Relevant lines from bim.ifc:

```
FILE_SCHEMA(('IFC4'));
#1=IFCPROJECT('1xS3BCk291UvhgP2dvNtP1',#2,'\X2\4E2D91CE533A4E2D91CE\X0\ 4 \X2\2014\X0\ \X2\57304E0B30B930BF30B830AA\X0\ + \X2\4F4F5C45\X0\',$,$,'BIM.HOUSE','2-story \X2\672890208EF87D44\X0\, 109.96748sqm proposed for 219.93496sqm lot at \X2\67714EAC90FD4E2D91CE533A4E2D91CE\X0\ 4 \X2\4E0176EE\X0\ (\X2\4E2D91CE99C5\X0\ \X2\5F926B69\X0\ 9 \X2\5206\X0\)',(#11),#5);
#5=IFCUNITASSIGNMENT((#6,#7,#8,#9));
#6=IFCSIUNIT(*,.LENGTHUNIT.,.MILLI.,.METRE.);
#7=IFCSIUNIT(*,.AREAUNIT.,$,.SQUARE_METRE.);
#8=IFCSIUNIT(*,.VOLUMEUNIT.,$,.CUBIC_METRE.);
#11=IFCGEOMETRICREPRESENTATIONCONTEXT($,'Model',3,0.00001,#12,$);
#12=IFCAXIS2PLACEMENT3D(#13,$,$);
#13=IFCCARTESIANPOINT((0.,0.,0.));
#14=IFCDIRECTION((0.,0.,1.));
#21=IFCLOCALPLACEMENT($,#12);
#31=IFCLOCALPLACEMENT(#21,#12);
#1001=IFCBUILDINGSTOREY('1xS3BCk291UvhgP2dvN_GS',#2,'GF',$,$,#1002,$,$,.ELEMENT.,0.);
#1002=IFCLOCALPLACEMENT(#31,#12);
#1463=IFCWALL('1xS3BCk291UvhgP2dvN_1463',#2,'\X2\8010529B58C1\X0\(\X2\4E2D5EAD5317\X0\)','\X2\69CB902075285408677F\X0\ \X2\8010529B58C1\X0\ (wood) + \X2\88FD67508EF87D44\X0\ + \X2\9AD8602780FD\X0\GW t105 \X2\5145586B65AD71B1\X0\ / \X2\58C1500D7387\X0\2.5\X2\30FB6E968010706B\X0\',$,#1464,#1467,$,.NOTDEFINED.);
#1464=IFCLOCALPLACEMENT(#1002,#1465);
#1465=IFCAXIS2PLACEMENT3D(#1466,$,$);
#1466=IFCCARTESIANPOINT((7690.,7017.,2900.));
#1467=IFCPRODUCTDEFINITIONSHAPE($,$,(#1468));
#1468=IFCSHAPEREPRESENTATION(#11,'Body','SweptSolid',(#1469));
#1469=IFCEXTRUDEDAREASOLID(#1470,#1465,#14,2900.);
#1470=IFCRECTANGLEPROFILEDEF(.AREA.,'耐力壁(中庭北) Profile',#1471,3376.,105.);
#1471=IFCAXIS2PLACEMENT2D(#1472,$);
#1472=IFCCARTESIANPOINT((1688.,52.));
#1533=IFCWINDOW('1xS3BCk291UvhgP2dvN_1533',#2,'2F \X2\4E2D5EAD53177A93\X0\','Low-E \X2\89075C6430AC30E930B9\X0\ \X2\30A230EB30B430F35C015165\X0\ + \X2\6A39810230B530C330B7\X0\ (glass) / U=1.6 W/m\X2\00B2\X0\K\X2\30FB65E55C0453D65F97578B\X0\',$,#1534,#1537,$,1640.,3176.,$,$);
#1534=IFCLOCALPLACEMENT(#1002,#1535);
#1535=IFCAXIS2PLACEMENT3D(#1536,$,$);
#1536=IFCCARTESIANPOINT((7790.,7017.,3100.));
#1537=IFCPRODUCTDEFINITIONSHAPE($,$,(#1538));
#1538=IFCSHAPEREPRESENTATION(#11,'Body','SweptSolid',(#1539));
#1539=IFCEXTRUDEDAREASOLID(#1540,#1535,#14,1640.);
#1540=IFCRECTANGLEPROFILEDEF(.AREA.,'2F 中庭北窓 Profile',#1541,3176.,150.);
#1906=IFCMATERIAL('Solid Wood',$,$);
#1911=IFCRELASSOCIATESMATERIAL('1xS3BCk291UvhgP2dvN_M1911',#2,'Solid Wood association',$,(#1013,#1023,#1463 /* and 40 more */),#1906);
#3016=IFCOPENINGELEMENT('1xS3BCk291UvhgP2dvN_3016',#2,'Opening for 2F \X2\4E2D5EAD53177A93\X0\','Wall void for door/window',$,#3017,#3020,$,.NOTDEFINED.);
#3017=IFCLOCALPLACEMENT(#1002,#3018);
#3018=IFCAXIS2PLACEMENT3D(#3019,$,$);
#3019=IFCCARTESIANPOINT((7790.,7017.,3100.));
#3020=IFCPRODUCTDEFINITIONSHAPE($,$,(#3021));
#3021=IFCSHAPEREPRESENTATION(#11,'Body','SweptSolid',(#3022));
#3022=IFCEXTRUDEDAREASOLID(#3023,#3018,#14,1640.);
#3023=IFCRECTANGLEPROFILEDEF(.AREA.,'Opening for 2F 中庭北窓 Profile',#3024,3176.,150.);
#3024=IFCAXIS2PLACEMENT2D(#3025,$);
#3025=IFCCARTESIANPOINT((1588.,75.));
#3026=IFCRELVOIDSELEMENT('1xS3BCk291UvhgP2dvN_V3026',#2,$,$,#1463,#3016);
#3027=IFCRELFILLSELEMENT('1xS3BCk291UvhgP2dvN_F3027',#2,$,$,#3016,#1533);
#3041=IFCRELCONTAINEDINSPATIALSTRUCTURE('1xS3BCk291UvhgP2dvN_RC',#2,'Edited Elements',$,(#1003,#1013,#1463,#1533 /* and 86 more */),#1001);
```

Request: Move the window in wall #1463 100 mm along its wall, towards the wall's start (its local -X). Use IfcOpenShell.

```python
import ifcopenshell
import ifcopenshell.api.geometry
import ifcopenshell.util.placement
import ifcopenshell.util.unit

model = ifcopenshell.open("bim.ifc")
unit_scale = ifcopenshell.util.unit.calculate_unit_scale(model)

window = model.by_guid("1xS3BCk291UvhgP2dvN_1533")
opening = window.FillsVoids[0].RelatingOpeningElement
wall = opening.VoidsElements[0].RelatingBuildingElement

wall_matrix = ifcopenshell.util.placement.get_local_placement(wall.ObjectPlacement)
shift = wall_matrix[:3, 0] * -0.1 / unit_scale
before = ifcopenshell.util.placement.get_local_placement(window.ObjectPlacement)[:3, 3].copy()

# The window is not placed relative to its opening, so move both.
for product in (opening, window):
    matrix = ifcopenshell.util.placement.get_local_placement(product.ObjectPlacement)
    matrix[:3, 3] += shift
    ifcopenshell.api.geometry.edit_object_placement(model, product=product, matrix=matrix, is_si=False)

after = ifcopenshell.util.placement.get_local_placement(window.ObjectPlacement)[:3, 3]
print("window moved by", (after - before).round(3) + 0.0)

model.write("bim_rev.ifc")
```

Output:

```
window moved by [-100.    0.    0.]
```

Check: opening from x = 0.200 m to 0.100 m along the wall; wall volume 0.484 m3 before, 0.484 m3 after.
